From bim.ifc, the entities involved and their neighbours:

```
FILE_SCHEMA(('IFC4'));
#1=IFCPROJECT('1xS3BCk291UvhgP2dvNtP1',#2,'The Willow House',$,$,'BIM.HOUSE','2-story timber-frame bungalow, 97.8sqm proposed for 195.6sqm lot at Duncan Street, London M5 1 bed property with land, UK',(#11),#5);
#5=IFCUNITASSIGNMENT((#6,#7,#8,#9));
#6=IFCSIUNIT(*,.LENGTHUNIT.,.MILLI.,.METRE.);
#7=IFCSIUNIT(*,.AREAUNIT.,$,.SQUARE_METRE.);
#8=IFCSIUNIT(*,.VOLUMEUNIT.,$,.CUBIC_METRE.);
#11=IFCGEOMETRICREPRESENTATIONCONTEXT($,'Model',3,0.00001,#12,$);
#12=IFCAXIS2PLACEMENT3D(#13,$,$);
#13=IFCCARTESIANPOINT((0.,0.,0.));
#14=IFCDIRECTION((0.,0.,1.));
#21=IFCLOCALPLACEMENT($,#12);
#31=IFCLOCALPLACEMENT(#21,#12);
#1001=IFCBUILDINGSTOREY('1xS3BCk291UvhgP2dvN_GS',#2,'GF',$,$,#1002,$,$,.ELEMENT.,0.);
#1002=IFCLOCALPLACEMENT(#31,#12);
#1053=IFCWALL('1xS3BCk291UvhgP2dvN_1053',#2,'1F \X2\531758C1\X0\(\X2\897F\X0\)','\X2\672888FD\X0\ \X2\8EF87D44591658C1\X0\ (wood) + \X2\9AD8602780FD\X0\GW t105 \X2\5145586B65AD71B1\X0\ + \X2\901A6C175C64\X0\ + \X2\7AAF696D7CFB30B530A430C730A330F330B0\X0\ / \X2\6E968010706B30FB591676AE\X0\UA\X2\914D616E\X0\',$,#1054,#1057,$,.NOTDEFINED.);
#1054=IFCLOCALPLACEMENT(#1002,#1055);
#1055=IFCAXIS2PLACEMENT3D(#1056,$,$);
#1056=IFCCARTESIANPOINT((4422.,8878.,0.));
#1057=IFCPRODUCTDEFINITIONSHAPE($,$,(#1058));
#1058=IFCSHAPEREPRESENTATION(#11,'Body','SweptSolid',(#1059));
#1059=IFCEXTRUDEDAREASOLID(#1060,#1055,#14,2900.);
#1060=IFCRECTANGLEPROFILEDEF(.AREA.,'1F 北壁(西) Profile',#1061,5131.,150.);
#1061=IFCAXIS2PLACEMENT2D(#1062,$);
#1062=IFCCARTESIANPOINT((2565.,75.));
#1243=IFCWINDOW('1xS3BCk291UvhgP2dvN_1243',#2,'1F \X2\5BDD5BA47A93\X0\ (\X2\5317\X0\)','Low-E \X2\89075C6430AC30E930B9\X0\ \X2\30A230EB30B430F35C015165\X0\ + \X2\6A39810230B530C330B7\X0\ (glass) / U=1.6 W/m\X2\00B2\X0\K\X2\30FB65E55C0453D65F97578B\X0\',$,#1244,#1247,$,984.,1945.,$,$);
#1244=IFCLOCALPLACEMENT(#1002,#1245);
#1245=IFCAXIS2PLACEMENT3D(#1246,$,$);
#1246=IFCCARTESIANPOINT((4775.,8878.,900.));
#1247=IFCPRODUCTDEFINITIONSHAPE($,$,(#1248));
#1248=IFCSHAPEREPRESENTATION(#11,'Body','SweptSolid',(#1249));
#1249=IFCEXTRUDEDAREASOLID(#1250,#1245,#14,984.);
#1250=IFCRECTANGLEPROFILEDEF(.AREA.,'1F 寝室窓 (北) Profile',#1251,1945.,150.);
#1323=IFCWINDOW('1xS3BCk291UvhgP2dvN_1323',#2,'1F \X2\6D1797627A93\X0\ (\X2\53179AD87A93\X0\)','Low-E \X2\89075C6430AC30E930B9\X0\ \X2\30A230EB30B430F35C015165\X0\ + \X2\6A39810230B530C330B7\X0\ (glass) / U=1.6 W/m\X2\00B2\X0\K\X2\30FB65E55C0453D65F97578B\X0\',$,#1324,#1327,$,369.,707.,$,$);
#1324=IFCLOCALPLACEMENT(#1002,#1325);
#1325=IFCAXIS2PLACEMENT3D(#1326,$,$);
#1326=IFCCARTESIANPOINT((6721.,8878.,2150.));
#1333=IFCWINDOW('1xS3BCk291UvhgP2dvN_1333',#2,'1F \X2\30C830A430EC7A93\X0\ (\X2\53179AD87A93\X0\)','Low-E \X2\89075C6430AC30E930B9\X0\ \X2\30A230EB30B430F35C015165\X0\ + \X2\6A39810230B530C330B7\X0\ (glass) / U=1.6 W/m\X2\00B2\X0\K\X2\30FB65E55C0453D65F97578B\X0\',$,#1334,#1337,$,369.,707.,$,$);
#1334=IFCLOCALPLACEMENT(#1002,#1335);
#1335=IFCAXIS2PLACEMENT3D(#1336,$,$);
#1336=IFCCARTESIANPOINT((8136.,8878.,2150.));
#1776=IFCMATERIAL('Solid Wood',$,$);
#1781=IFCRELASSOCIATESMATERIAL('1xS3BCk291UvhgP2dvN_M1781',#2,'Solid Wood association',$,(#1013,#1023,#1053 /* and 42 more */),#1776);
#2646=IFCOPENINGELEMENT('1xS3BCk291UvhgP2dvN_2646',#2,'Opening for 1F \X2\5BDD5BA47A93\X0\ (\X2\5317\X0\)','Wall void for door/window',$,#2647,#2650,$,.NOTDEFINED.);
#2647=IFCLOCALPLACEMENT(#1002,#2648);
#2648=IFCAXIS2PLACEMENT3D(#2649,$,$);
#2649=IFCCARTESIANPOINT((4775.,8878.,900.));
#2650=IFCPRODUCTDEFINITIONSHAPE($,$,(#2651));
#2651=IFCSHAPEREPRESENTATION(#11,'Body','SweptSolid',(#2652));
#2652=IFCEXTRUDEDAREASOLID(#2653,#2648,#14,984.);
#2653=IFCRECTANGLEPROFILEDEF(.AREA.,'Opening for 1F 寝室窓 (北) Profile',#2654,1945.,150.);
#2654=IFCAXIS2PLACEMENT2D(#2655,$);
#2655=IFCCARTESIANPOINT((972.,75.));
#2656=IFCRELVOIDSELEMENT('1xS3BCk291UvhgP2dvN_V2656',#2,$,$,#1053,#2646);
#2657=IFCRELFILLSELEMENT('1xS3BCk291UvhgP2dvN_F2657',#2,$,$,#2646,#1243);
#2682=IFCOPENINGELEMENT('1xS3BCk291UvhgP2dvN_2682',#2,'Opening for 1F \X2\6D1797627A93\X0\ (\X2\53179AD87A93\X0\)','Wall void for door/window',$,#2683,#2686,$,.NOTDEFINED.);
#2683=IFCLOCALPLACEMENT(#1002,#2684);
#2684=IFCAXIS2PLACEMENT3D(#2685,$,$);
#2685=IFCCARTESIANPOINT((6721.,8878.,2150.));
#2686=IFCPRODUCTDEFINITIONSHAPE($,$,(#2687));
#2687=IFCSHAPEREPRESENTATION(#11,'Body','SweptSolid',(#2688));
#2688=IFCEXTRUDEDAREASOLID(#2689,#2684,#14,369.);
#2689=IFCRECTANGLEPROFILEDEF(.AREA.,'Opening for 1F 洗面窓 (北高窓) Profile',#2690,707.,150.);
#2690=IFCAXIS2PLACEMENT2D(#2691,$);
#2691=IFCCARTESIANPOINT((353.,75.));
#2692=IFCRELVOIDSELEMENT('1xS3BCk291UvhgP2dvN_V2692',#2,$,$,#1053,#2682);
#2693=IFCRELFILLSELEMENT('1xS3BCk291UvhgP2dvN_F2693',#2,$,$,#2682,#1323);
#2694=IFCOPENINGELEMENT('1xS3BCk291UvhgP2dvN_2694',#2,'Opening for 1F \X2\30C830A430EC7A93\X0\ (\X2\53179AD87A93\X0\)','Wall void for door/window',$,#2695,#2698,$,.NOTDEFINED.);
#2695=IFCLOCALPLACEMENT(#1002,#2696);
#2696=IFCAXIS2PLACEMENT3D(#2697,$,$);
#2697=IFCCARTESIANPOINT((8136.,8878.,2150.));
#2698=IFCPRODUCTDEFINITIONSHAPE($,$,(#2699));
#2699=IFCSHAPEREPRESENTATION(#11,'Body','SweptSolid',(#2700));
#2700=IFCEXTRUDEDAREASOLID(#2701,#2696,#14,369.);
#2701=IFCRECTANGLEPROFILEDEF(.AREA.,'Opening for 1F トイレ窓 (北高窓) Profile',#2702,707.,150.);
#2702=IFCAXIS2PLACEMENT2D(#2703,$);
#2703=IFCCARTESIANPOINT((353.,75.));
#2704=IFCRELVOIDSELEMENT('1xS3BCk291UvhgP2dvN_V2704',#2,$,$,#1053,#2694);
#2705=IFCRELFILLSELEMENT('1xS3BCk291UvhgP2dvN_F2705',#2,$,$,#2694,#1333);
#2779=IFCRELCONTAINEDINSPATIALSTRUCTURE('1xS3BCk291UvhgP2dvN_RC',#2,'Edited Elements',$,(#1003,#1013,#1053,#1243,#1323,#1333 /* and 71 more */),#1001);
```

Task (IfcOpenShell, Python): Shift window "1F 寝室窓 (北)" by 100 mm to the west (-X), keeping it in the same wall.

```python
import ifcopenshell
import ifcopenshell.api.geometry
import ifcopenshell.util.placement
import ifcopenshell.util.unit

model = ifcopenshell.open("bim.ifc")
unit_scale = ifcopenshell.util.unit.calculate_unit_scale(model)

window = model.by_guid("1xS3BCk291UvhgP2dvN_1243")
opening = window.FillsVoids[0].RelatingOpeningElement
wall = opening.VoidsElements[0].RelatingBuildingElement

wall_matrix = ifcopenshell.util.placement.get_local_placement(wall.ObjectPlacement)
shift = wall_matrix[:3, 0] * -0.1 / unit_scale
before = ifcopenshell.util.placement.get_local_placement(window.ObjectPlacement)[:3, 3].copy()

# The window is not placed relative to its opening, so move both.
for product in (opening, window):
    matrix = ifcopenshell.util.placement.get_local_placement(product.ObjectPlacement)
    matrix[:3, 3] += shift
    ifcopenshell.api.geometry.edit_object_placement(model, product=product, matrix=matrix, is_si=False)

after = ifcopenshell.util.placement.get_local_placement(window.ObjectPlacement)[:3, 3]
print("window moved by", (after - before).round(3) + 0.0)

model.write("bim_edited.ifc")
```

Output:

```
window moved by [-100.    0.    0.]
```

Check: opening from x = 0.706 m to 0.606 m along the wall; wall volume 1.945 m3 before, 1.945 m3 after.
